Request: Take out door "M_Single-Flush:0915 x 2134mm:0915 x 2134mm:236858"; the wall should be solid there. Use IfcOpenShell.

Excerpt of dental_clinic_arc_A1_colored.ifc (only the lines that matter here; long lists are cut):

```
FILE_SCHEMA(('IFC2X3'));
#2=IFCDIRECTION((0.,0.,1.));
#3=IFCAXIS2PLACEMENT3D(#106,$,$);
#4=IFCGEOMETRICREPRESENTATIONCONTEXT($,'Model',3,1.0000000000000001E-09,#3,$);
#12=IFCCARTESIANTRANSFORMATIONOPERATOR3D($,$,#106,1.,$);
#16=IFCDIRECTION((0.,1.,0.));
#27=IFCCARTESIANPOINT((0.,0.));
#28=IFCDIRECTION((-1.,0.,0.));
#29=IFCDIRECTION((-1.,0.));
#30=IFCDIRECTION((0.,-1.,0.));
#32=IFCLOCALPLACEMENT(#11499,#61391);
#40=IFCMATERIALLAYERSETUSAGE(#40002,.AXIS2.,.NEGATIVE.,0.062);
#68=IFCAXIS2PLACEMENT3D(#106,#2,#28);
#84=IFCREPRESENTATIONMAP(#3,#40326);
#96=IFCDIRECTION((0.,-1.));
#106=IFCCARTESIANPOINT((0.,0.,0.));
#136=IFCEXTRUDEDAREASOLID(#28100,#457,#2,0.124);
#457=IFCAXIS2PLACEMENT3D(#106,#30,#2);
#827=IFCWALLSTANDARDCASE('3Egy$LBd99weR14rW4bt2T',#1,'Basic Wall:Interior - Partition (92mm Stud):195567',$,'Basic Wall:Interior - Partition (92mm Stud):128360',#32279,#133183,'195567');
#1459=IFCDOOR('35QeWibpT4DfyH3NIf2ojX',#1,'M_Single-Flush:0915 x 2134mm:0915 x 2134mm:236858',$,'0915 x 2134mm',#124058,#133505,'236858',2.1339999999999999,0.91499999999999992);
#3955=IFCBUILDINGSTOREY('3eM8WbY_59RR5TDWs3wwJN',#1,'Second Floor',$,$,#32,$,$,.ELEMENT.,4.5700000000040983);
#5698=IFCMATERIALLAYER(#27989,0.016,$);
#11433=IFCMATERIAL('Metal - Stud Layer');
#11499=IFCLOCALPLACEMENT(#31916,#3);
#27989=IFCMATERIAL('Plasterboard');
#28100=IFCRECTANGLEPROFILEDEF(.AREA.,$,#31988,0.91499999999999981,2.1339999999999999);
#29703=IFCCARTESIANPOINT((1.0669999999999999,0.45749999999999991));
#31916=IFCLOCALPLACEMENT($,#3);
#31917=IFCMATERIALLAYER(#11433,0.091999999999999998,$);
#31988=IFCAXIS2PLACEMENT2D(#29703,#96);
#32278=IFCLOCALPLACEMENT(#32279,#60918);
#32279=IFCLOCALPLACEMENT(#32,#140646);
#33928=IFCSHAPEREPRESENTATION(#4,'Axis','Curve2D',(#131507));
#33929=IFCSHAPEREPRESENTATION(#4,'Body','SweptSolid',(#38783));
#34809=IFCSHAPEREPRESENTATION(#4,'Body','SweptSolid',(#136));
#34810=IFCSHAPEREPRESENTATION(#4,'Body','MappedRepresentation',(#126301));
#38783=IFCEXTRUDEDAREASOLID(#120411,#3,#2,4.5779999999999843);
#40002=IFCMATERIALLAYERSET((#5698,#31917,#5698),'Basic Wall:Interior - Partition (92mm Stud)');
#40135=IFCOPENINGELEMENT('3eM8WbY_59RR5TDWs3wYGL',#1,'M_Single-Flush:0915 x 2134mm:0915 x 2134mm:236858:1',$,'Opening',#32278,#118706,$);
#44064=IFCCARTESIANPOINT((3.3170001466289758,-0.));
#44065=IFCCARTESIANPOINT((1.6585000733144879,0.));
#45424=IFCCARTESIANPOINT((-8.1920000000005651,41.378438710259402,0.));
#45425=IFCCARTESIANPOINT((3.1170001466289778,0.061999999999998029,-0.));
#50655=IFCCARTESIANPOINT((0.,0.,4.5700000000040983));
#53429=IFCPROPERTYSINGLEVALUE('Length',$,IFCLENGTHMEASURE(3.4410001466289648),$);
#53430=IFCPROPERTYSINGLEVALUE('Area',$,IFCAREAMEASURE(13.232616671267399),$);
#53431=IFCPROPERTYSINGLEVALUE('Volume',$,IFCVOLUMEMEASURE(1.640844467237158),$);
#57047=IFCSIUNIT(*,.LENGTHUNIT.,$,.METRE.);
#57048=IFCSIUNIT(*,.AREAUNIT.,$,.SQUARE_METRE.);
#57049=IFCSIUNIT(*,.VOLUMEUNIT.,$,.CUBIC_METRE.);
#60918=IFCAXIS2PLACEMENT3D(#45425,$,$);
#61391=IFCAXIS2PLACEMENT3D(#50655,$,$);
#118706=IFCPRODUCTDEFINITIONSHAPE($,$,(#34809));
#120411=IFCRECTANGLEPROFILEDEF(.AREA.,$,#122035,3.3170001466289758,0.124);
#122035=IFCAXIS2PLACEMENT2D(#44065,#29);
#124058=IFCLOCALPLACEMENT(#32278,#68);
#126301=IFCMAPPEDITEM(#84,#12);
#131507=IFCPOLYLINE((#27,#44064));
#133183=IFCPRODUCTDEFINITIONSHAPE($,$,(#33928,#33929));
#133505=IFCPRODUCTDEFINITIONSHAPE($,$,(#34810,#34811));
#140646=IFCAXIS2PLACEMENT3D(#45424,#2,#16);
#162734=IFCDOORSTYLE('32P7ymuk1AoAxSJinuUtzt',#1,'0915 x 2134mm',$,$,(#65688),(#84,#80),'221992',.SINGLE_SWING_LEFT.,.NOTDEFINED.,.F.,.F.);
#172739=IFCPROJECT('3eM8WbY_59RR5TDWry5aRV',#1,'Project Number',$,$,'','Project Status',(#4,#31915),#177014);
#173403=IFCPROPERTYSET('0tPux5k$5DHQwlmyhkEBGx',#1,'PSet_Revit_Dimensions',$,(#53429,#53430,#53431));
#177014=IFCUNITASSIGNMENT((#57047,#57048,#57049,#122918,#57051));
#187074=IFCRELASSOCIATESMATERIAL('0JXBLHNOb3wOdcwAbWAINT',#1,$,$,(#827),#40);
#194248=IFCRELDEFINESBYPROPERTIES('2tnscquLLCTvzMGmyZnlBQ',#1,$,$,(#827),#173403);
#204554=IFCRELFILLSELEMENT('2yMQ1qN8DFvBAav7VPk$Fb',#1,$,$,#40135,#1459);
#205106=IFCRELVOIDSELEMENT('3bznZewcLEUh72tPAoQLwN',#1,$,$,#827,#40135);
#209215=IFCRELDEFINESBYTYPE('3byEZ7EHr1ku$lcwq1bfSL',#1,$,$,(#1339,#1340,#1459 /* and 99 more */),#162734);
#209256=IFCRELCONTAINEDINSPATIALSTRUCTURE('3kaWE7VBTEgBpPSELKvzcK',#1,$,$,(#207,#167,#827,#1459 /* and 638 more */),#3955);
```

```python
import ifcopenshell
import ifcopenshell.api.feature
import ifcopenshell.api.pset
import ifcopenshell.api.root
import ifcopenshell.geom
import ifcopenshell.util.element
import ifcopenshell.util.shape
import ifcopenshell.util.unit

model = ifcopenshell.open("dental_clinic_arc_A1_colored.ifc")
area_scale = ifcopenshell.util.unit.calculate_unit_scale(model, "AREAUNIT")
volume_scale = ifcopenshell.util.unit.calculate_unit_scale(model, "VOLUMEUNIT")
settings = ifcopenshell.geom.settings()


def volume(element):
    """Net volume in cubic metres, openings subtracted."""
    shape = ifcopenshell.geom.create_shape(settings, element)
    return ifcopenshell.util.shape.get_volume(shape.geometry)


door = model.by_guid("35QeWibpT4DfyH3NIf2ojX")
opening = door.FillsVoids[0].RelatingOpeningElement
wall = opening.VoidsElements[0].RelatingBuildingElement
before = volume(wall)

ifcopenshell.api.root.remove_product(model, product=door)
ifcopenshell.api.feature.remove_feature(model, feature=opening)

after = volume(wall)
thickness = 0.124  # wall thickness in metres

# Update the wall's stored quantities.
pset = model.by_id(ifcopenshell.util.element.get_pset(wall, "PSet_Revit_Dimensions", should_inherit=False)["id"])
ifcopenshell.api.pset.edit_pset(model, pset=pset, properties={
    "Area": model.create_entity("IfcAreaMeasure", after / thickness / area_scale),
    "Volume": model.create_entity("IfcVolumeMeasure", after / volume_scale),
})

print(f"wall volume {before:.3f} -> {after:.3f} m3")

model.write("dental_clinic_arc_A1_colored_rev.ifc")
```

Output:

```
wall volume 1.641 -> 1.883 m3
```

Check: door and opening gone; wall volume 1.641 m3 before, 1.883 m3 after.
